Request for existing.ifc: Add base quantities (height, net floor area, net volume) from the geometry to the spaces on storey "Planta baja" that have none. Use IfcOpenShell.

First a look at what the model holds.

```python
import ifcopenshell
import ifcopenshell.util.element
import ifcopenshell.util.unit

model = ifcopenshell.open("existing.ifc")
print(model.schema)
for unit_type in ("LENGTHUNIT", "AREAUNIT", "VOLUMEUNIT"):
    print(unit_type, ifcopenshell.util.unit.calculate_unit_scale(model, unit_type))
storey = next(s for s in model.by_type("IfcBuildingStorey") if s.Name == "Planta baja")
spaces = [e for e in ifcopenshell.util.element.get_decomposition(storey) if e.is_a("IfcSpace")]
for e in sorted(spaces, key=lambda e: e.id()):
    print(e.id(), e.is_a(), e.Name, list(ifcopenshell.util.element.get_psets(e, qtos_only=True)), sep=" | ")
```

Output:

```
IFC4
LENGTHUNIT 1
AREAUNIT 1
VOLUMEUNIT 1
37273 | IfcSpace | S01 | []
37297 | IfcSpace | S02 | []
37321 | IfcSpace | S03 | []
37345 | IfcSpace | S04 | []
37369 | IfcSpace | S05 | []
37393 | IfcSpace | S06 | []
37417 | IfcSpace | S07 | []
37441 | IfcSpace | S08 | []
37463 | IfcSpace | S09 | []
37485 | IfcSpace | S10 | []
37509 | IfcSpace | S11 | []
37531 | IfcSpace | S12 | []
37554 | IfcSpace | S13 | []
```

```python
import ifcopenshell
import ifcopenshell.api.pset
import ifcopenshell.geom
import ifcopenshell.util.element
import ifcopenshell.util.shape
import ifcopenshell.util.unit

model = ifcopenshell.open("existing.ifc")
unit_scale = ifcopenshell.util.unit.calculate_unit_scale(model)
area_scale = ifcopenshell.util.unit.calculate_unit_scale(model, "AREAUNIT")
volume_scale = ifcopenshell.util.unit.calculate_unit_scale(model, "VOLUMEUNIT")
settings = ifcopenshell.geom.settings()

storey = next(s for s in model.by_type("IfcBuildingStorey") if s.Name == "Planta baja")
spaces = [e for e in ifcopenshell.util.element.get_decomposition(storey) if e.is_a("IfcSpace")]

for e in sorted(spaces, key=lambda e: e.id()):
    if ifcopenshell.util.element.get_psets(e, qtos_only=True, should_inherit=False):
        continue
    # Geometry comes back in metres, in the element's own axes.
    shape = ifcopenshell.geom.create_shape(settings, e)
    values = {
        "Height": ifcopenshell.util.shape.get_z(shape.geometry) / unit_scale,
        "NetFloorArea": ifcopenshell.util.shape.get_footprint_area(shape.geometry) / area_scale,
        "NetVolume": ifcopenshell.util.shape.get_volume(shape.geometry) / volume_scale,
    }
    qto = ifcopenshell.api.pset.add_qto(model, product=e, name="Qto_SpaceBaseQuantities")
    ifcopenshell.api.pset.edit_qto(model, qto=qto, properties=values)
    print(e.id(), {k: round(v, 3) for k, v in values.items()})

model.write("existing_edited.ifc")
```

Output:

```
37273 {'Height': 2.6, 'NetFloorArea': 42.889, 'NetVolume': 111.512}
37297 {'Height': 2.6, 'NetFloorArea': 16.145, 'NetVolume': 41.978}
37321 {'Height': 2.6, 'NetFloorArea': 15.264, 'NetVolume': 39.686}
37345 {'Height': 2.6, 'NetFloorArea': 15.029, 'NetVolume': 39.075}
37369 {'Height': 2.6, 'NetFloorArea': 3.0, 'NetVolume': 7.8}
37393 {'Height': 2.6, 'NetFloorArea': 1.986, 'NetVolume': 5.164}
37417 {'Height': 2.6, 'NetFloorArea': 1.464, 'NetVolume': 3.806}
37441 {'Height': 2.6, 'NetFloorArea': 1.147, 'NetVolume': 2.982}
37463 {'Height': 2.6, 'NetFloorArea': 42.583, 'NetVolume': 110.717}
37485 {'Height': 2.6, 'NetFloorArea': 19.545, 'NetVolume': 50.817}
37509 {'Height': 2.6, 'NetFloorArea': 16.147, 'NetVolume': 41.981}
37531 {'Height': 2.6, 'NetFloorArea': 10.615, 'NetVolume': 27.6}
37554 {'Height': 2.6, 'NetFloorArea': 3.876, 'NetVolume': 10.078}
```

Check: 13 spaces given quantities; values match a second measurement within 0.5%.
